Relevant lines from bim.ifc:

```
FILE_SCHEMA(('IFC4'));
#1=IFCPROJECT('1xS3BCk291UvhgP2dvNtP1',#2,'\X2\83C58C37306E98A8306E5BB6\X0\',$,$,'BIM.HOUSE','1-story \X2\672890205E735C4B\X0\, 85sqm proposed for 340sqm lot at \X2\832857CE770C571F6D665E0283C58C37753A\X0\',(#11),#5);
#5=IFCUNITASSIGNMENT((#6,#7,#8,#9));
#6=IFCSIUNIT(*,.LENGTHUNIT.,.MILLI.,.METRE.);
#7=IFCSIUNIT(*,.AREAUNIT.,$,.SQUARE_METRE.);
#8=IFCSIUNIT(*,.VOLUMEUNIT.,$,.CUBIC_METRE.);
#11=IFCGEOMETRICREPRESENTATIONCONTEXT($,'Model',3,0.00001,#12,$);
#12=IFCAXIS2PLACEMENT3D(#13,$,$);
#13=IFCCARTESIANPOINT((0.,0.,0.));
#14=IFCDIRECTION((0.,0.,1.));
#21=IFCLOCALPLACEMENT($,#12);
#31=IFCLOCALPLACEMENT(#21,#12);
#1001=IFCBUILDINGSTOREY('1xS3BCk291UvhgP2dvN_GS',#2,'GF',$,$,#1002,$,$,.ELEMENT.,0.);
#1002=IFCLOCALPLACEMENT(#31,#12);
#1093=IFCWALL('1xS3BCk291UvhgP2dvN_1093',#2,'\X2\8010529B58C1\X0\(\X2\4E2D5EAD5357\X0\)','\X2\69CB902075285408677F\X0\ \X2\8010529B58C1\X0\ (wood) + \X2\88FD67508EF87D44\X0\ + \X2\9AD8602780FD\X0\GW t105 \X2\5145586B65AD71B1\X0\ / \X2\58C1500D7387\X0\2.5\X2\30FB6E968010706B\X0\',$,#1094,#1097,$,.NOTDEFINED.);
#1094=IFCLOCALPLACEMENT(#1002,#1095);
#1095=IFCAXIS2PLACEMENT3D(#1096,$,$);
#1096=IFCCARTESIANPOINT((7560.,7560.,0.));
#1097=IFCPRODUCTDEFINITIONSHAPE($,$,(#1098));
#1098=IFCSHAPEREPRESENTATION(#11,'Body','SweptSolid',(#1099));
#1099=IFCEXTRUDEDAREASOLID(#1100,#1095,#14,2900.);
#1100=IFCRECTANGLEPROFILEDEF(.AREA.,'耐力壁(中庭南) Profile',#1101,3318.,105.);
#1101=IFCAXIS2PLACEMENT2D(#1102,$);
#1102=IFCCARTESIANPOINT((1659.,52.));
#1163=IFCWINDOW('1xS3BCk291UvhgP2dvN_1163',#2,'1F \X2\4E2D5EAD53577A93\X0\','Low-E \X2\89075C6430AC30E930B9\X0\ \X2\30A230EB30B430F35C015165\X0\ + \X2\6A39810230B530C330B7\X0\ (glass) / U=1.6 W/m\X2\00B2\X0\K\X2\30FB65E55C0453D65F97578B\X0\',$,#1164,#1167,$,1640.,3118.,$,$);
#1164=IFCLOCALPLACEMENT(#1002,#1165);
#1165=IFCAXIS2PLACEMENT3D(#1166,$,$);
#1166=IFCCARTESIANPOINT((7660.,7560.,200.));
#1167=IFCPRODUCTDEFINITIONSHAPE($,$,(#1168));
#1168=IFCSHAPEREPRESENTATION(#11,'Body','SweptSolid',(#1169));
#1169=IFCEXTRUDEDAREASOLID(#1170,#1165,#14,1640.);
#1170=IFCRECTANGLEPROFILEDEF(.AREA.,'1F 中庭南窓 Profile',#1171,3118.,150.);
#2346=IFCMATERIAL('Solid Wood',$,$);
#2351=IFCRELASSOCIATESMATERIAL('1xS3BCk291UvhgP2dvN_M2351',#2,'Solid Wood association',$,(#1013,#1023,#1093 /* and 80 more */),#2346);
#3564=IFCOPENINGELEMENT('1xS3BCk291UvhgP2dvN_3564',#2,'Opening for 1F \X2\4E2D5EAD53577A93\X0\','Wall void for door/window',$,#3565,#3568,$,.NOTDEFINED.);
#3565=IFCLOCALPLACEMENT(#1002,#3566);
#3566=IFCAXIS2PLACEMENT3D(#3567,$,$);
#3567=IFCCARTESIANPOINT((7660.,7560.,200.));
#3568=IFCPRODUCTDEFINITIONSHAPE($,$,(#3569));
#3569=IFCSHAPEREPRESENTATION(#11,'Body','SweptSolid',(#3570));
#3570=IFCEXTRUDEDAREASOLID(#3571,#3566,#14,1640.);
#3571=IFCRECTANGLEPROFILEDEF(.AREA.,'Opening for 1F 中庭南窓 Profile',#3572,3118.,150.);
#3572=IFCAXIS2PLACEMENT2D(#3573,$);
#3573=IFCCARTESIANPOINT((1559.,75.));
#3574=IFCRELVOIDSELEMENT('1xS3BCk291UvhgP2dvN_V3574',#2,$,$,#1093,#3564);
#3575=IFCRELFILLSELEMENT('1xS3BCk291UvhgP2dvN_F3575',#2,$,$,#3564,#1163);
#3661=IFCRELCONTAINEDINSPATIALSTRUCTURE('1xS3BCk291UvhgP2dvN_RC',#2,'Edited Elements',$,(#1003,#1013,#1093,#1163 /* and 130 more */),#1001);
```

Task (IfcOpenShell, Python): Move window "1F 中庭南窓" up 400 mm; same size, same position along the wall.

```python
import numpy as np
import ifcopenshell
import ifcopenshell.api.geometry
import ifcopenshell.util.placement
import ifcopenshell.util.unit

model = ifcopenshell.open("bim.ifc")
unit_scale = ifcopenshell.util.unit.calculate_unit_scale(model)

window = model.by_guid("1xS3BCk291UvhgP2dvN_1163")
opening = window.FillsVoids[0].RelatingOpeningElement
dz = 0.4 / unit_scale

shift = np.array([0.0, 0.0, dz])
# The window is not placed relative to its opening, so move both.
for product in (opening, window):
    matrix = ifcopenshell.util.placement.get_local_placement(product.ObjectPlacement)
    matrix[:3, 3] += shift
    ifcopenshell.api.geometry.edit_object_placement(model, product=product, matrix=matrix, is_si=False)

print(f"moved by {dz * unit_scale:+.3f} m")

model.write("bim-out.ifc")
```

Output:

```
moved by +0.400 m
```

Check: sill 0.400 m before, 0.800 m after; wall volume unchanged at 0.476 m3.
